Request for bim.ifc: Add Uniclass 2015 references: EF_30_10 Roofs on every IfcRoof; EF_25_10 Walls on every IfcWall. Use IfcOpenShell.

First a look at what the model holds.

```python
import ifcopenshell

model = ifcopenshell.open("bim.ifc")
print(model.schema)
print("classifications:", [c.Name for c in model.by_type("IfcClassification")])
for ifc_class in ("IfcDoor", "IfcRoof", "IfcStair", "IfcWall", "IfcWindow"):
    print(ifc_class, len(model.by_type(ifc_class)))
```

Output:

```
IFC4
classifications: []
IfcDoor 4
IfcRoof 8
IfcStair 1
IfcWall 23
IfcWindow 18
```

```python
import ifcopenshell
import ifcopenshell.api.classification

model = ifcopenshell.open("bim.ifc")

system = ifcopenshell.api.classification.add_classification(model, classification="Uniclass 2015")

codes = {
    "IfcRoof": ("EF_30_10", "Roofs"),
    "IfcWall": ("EF_25_10", "Walls"),
}
for ifc_class, (code, name) in codes.items():
    products = model.by_type(ifc_class)
    ifcopenshell.api.classification.add_reference(
        model, products=products, classification=system, identification=code, name=name
    )
    print(code, len(products))

model.write("bim_updated.ifc")
```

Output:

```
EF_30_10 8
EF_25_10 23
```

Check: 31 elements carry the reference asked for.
